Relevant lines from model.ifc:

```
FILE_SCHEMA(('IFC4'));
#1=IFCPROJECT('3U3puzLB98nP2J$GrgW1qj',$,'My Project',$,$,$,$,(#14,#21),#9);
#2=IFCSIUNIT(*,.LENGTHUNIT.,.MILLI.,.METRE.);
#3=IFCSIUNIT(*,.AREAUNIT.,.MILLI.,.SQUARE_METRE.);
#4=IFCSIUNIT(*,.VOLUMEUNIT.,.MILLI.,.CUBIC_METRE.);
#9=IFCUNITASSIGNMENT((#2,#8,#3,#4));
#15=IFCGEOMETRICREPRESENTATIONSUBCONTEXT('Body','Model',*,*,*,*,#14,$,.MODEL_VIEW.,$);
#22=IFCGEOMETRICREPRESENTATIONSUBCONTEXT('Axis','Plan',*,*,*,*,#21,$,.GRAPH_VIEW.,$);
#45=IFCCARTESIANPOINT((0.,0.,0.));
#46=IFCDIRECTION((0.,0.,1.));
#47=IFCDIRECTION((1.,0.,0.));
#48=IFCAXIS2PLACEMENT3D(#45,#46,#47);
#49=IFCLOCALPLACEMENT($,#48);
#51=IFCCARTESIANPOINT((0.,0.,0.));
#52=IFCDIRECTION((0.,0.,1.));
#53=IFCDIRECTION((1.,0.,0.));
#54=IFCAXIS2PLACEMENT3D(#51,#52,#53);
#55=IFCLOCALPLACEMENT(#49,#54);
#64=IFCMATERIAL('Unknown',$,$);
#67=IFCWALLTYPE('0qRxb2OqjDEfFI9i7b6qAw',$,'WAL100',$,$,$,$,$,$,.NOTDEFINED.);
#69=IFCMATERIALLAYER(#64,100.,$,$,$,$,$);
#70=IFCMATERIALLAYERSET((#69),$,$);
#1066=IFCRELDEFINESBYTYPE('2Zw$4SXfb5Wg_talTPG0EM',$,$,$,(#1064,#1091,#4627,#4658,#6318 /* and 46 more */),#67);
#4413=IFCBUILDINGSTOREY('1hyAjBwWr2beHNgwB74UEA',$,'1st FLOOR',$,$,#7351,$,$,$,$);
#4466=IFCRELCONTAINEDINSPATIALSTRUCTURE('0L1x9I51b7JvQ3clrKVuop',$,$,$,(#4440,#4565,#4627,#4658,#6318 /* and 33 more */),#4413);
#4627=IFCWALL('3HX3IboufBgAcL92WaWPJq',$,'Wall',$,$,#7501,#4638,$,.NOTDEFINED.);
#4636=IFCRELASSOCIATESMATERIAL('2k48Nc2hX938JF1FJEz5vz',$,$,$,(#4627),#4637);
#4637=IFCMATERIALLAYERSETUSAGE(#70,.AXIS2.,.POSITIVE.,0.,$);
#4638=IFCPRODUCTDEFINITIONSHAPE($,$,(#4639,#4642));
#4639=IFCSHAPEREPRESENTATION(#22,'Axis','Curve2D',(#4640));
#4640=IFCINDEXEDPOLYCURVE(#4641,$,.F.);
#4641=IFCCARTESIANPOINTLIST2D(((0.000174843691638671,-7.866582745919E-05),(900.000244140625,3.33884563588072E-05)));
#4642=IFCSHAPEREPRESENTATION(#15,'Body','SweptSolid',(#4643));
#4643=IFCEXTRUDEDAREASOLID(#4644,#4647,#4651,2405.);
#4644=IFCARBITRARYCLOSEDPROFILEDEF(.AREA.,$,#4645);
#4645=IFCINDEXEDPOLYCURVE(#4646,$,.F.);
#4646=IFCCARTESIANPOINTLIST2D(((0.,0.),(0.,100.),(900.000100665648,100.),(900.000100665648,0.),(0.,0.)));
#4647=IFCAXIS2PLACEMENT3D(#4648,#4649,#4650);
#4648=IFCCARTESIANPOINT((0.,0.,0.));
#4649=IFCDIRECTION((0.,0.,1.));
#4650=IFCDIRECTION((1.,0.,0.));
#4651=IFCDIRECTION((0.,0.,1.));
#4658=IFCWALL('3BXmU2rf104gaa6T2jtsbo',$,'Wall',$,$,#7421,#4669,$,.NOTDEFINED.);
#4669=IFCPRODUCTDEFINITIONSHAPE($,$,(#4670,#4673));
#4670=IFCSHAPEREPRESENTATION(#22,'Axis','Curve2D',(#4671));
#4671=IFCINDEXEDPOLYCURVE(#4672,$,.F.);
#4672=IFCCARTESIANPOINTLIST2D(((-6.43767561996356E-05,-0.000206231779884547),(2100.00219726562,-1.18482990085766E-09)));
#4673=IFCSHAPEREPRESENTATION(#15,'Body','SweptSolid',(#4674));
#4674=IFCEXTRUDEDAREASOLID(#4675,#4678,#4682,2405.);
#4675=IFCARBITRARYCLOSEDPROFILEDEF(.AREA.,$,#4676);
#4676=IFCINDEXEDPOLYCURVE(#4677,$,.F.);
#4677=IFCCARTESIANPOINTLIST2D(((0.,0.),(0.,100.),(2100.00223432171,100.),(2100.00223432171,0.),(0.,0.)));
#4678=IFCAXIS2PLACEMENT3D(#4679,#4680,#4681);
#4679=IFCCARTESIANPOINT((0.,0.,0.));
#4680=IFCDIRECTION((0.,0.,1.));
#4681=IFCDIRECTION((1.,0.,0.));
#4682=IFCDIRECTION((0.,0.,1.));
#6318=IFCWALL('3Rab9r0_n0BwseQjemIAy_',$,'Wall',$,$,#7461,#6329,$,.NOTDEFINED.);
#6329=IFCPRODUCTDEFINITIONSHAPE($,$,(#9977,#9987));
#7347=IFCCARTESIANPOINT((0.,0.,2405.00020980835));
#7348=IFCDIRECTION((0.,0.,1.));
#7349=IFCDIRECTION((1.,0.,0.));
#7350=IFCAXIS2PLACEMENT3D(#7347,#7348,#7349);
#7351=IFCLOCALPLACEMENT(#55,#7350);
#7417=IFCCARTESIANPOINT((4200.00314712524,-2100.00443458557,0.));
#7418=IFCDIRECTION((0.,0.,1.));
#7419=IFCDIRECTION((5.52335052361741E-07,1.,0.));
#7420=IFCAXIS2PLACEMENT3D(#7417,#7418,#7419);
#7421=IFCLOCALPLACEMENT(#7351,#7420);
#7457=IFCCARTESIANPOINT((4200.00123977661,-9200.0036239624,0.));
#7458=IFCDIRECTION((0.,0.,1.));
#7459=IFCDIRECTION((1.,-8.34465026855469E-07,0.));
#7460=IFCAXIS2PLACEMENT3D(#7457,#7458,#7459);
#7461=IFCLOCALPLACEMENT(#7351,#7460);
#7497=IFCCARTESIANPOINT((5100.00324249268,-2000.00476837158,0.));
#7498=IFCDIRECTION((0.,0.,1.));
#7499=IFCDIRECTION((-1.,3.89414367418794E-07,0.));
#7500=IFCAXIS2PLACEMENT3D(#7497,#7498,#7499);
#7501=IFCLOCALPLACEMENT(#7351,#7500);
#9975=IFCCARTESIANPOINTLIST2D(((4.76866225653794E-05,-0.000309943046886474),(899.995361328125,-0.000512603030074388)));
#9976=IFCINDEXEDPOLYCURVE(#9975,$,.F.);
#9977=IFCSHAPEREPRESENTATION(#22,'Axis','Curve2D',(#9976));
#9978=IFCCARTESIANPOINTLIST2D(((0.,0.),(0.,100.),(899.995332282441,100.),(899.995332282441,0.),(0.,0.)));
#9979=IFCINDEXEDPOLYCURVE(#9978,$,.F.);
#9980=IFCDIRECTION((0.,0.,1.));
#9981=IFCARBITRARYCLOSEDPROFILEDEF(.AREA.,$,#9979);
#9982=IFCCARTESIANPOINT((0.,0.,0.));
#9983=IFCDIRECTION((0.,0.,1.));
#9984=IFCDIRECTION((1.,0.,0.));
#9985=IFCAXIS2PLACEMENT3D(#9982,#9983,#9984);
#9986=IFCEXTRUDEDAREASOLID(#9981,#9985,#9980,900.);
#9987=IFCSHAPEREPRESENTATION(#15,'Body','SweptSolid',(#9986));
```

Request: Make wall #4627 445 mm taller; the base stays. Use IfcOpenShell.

```python
import ifcopenshell
import ifcopenshell.geom
import ifcopenshell.util.representation
import ifcopenshell.util.shape
import ifcopenshell.util.unit

model = ifcopenshell.open("model.ifc")
unit_scale = ifcopenshell.util.unit.calculate_unit_scale(model)
settings = ifcopenshell.geom.settings()


def volume(element):
    """Net volume in cubic metres, openings subtracted."""
    shape = ifcopenshell.geom.create_shape(settings, element)
    return ifcopenshell.util.shape.get_volume(shape.geometry)


wall = model.by_guid("3HX3IboufBgAcL92WaWPJq")
before = volume(wall)

body = ifcopenshell.util.representation.get_representation(wall, "Model", "Body")
solid = body.Items[0]
old_height = solid.Depth
solid.Depth += 0.445 / unit_scale
after = volume(wall)

print(f"height {old_height:g} -> {solid.Depth:g}, volume {before:.3f} -> {after:.3f} m3")

model.write("model_v2.ifc")
```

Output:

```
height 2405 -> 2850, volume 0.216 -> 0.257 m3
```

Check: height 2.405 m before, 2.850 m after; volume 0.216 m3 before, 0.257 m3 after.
